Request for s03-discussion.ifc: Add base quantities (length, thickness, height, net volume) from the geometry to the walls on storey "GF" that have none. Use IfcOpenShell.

First a look at what the model holds.

```python
import ifcopenshell
import ifcopenshell.util.element
import ifcopenshell.util.unit

model = ifcopenshell.open("s03-discussion.ifc")
print(model.schema)
for unit_type in ("LENGTHUNIT", "AREAUNIT", "VOLUMEUNIT"):
    print(unit_type, ifcopenshell.util.unit.calculate_unit_scale(model, unit_type))
storey = next(s for s in model.by_type("IfcBuildingStorey") if s.Name == "GF")
walls = [e for e in ifcopenshell.util.element.get_decomposition(storey) if e.is_a("IfcWall")]
for e in sorted(walls, key=lambda e: e.id()):
    print(e.id(), e.is_a(), e.Name, list(ifcopenshell.util.element.get_psets(e, qtos_only=True)), sep=" | ")
```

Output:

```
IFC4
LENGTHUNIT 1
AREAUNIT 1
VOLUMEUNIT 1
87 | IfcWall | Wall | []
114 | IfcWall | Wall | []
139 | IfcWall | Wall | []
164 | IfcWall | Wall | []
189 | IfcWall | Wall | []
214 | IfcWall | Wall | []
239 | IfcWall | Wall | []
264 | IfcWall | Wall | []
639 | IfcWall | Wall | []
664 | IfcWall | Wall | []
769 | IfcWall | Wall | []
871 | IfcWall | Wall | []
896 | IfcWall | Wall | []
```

```python
import ifcopenshell
import ifcopenshell.api.pset
import ifcopenshell.geom
import ifcopenshell.util.element
import ifcopenshell.util.shape
import ifcopenshell.util.unit

model = ifcopenshell.open("s03-discussion.ifc")
unit_scale = ifcopenshell.util.unit.calculate_unit_scale(model)
volume_scale = ifcopenshell.util.unit.calculate_unit_scale(model, "VOLUMEUNIT")
settings = ifcopenshell.geom.settings()

storey = next(s for s in model.by_type("IfcBuildingStorey") if s.Name == "GF")
walls = [e for e in ifcopenshell.util.element.get_decomposition(storey) if e.is_a("IfcWall")]

for e in sorted(walls, key=lambda e: e.id()):
    if ifcopenshell.util.element.get_psets(e, qtos_only=True, should_inherit=False):
        continue
    # Geometry comes back in metres, in the element's own axes.
    shape = ifcopenshell.geom.create_shape(settings, e)
    values = {
        "Length": ifcopenshell.util.shape.get_x(shape.geometry) / unit_scale,
        "Width": ifcopenshell.util.shape.get_y(shape.geometry) / unit_scale,
        "Height": ifcopenshell.util.shape.get_z(shape.geometry) / unit_scale,
        "NetVolume": ifcopenshell.util.shape.get_volume(shape.geometry) / volume_scale,
    }
    qto = ifcopenshell.api.pset.add_qto(model, product=e, name="Qto_WallBaseQuantities")
    ifcopenshell.api.pset.edit_qto(model, qto=qto, properties=values)
    print(e.id(), {k: round(v, 3) for k, v in values.items()})

model.write("s03-discussion-out.ifc")
```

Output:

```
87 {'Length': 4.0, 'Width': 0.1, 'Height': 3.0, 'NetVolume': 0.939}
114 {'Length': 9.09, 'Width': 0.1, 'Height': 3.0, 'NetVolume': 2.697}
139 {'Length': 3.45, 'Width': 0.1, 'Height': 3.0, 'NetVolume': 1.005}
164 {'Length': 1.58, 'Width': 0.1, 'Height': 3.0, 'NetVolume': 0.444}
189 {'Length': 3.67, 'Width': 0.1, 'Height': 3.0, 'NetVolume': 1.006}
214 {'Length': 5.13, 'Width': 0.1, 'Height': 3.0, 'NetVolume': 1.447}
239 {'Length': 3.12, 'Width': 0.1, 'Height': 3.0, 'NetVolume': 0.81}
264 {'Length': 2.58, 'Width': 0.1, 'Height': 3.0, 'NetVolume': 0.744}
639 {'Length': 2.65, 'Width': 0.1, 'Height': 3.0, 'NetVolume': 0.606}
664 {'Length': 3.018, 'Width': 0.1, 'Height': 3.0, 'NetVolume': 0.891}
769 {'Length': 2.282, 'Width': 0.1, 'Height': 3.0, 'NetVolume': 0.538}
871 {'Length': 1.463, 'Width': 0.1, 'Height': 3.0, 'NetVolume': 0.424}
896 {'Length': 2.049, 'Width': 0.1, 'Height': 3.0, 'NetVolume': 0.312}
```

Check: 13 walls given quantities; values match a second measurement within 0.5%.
